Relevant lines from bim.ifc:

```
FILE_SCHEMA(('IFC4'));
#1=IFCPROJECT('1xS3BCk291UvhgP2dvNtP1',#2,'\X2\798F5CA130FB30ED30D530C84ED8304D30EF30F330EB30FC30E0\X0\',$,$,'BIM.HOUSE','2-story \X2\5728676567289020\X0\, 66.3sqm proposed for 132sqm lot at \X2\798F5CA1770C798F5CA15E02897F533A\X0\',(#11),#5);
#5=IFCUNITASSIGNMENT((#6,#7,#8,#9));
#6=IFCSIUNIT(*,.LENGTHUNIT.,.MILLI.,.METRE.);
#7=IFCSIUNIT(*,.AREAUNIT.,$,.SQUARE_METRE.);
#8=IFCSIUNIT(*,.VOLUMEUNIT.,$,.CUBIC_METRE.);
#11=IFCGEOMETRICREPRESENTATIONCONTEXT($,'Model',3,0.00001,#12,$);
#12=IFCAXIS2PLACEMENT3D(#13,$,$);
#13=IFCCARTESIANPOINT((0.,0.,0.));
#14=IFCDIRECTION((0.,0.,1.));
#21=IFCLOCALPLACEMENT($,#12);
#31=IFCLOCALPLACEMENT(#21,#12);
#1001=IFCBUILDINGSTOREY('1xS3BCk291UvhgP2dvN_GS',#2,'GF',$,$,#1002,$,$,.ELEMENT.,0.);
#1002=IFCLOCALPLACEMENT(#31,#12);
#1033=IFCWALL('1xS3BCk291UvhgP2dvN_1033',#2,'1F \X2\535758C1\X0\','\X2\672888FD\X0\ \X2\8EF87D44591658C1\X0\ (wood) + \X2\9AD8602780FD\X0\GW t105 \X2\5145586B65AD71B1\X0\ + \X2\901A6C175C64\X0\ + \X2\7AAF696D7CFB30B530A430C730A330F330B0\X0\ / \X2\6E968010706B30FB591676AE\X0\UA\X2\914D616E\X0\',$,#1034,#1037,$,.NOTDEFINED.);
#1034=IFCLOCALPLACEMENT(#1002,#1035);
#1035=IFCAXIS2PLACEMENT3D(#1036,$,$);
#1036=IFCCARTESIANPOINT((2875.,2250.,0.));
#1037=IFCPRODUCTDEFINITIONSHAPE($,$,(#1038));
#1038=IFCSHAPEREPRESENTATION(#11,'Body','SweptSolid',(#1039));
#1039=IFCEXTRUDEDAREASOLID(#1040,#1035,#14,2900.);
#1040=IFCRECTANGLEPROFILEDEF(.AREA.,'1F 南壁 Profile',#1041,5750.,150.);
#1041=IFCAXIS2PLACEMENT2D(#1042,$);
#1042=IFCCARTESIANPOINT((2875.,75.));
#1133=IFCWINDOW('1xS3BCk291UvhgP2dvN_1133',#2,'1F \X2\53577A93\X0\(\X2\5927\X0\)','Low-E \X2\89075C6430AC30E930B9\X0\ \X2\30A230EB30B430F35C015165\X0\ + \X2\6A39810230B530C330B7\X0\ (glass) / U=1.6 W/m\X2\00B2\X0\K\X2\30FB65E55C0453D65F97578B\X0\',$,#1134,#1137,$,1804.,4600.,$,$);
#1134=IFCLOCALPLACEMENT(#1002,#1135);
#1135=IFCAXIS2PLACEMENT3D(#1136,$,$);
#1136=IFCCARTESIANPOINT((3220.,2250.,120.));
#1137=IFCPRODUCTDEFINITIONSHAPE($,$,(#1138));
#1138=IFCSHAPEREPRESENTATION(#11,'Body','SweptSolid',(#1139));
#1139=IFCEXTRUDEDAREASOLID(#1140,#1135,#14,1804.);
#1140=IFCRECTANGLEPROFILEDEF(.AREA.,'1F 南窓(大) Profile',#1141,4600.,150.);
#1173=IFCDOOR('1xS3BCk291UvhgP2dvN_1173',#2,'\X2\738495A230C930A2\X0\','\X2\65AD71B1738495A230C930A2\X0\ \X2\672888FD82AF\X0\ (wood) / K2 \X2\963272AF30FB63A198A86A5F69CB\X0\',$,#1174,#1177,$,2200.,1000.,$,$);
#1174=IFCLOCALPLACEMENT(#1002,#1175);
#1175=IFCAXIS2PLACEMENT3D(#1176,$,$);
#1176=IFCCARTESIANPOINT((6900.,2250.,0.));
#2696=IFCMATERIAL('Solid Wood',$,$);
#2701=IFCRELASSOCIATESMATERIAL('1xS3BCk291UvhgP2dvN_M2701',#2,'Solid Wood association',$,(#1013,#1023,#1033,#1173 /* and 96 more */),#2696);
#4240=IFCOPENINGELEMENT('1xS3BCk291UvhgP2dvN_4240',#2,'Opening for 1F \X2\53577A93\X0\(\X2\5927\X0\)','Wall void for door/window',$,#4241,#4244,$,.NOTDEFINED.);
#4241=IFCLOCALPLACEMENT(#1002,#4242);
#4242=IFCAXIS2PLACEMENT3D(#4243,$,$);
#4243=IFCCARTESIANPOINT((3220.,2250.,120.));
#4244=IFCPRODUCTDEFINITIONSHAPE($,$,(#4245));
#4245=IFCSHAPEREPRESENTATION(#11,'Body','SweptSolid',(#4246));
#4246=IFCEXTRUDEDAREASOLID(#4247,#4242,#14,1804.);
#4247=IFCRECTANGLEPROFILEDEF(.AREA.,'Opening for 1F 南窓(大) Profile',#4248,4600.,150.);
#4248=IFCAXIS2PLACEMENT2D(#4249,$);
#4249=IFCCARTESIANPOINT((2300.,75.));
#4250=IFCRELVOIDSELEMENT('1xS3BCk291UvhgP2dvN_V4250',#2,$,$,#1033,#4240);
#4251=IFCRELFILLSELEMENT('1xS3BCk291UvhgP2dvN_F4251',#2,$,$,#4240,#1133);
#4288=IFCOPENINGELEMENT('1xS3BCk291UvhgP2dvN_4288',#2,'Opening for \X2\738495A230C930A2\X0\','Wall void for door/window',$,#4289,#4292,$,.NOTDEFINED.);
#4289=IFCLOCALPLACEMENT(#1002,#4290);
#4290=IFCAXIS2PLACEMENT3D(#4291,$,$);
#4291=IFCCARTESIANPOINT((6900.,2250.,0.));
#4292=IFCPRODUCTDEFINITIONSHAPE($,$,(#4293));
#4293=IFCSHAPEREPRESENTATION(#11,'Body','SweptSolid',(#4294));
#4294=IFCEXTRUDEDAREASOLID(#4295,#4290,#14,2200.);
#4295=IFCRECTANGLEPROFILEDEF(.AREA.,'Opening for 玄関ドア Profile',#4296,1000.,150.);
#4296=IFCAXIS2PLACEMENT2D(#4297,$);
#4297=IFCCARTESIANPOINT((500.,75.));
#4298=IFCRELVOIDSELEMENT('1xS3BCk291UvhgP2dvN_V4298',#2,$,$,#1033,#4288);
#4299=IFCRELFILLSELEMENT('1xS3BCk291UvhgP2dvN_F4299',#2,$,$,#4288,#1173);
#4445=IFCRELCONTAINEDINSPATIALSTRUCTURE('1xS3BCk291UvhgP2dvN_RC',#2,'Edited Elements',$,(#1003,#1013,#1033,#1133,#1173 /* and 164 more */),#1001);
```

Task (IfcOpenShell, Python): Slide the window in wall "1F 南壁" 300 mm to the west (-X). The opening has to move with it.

```python
import ifcopenshell
import ifcopenshell.api.geometry
import ifcopenshell.util.placement
import ifcopenshell.util.unit

model = ifcopenshell.open("bim.ifc")
unit_scale = ifcopenshell.util.unit.calculate_unit_scale(model)

window = model.by_id(1133)
opening = window.FillsVoids[0].RelatingOpeningElement
wall = opening.VoidsElements[0].RelatingBuildingElement

wall_matrix = ifcopenshell.util.placement.get_local_placement(wall.ObjectPlacement)
shift = wall_matrix[:3, 0] * -0.3 / unit_scale
before = ifcopenshell.util.placement.get_local_placement(window.ObjectPlacement)[:3, 3].copy()

# The window is not placed relative to its opening, so move both.
for product in (opening, window):
    matrix = ifcopenshell.util.placement.get_local_placement(product.ObjectPlacement)
    matrix[:3, 3] += shift
    ifcopenshell.api.geometry.edit_object_placement(model, product=product, matrix=matrix, is_si=False)

after = ifcopenshell.util.placement.get_local_placement(window.ObjectPlacement)[:3, 3]
print("window moved by", (after - before).round(3) + 0.0)

model.write("bim_edited.ifc")
```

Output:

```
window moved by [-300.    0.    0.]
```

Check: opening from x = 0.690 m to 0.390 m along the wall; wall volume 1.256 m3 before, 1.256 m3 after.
